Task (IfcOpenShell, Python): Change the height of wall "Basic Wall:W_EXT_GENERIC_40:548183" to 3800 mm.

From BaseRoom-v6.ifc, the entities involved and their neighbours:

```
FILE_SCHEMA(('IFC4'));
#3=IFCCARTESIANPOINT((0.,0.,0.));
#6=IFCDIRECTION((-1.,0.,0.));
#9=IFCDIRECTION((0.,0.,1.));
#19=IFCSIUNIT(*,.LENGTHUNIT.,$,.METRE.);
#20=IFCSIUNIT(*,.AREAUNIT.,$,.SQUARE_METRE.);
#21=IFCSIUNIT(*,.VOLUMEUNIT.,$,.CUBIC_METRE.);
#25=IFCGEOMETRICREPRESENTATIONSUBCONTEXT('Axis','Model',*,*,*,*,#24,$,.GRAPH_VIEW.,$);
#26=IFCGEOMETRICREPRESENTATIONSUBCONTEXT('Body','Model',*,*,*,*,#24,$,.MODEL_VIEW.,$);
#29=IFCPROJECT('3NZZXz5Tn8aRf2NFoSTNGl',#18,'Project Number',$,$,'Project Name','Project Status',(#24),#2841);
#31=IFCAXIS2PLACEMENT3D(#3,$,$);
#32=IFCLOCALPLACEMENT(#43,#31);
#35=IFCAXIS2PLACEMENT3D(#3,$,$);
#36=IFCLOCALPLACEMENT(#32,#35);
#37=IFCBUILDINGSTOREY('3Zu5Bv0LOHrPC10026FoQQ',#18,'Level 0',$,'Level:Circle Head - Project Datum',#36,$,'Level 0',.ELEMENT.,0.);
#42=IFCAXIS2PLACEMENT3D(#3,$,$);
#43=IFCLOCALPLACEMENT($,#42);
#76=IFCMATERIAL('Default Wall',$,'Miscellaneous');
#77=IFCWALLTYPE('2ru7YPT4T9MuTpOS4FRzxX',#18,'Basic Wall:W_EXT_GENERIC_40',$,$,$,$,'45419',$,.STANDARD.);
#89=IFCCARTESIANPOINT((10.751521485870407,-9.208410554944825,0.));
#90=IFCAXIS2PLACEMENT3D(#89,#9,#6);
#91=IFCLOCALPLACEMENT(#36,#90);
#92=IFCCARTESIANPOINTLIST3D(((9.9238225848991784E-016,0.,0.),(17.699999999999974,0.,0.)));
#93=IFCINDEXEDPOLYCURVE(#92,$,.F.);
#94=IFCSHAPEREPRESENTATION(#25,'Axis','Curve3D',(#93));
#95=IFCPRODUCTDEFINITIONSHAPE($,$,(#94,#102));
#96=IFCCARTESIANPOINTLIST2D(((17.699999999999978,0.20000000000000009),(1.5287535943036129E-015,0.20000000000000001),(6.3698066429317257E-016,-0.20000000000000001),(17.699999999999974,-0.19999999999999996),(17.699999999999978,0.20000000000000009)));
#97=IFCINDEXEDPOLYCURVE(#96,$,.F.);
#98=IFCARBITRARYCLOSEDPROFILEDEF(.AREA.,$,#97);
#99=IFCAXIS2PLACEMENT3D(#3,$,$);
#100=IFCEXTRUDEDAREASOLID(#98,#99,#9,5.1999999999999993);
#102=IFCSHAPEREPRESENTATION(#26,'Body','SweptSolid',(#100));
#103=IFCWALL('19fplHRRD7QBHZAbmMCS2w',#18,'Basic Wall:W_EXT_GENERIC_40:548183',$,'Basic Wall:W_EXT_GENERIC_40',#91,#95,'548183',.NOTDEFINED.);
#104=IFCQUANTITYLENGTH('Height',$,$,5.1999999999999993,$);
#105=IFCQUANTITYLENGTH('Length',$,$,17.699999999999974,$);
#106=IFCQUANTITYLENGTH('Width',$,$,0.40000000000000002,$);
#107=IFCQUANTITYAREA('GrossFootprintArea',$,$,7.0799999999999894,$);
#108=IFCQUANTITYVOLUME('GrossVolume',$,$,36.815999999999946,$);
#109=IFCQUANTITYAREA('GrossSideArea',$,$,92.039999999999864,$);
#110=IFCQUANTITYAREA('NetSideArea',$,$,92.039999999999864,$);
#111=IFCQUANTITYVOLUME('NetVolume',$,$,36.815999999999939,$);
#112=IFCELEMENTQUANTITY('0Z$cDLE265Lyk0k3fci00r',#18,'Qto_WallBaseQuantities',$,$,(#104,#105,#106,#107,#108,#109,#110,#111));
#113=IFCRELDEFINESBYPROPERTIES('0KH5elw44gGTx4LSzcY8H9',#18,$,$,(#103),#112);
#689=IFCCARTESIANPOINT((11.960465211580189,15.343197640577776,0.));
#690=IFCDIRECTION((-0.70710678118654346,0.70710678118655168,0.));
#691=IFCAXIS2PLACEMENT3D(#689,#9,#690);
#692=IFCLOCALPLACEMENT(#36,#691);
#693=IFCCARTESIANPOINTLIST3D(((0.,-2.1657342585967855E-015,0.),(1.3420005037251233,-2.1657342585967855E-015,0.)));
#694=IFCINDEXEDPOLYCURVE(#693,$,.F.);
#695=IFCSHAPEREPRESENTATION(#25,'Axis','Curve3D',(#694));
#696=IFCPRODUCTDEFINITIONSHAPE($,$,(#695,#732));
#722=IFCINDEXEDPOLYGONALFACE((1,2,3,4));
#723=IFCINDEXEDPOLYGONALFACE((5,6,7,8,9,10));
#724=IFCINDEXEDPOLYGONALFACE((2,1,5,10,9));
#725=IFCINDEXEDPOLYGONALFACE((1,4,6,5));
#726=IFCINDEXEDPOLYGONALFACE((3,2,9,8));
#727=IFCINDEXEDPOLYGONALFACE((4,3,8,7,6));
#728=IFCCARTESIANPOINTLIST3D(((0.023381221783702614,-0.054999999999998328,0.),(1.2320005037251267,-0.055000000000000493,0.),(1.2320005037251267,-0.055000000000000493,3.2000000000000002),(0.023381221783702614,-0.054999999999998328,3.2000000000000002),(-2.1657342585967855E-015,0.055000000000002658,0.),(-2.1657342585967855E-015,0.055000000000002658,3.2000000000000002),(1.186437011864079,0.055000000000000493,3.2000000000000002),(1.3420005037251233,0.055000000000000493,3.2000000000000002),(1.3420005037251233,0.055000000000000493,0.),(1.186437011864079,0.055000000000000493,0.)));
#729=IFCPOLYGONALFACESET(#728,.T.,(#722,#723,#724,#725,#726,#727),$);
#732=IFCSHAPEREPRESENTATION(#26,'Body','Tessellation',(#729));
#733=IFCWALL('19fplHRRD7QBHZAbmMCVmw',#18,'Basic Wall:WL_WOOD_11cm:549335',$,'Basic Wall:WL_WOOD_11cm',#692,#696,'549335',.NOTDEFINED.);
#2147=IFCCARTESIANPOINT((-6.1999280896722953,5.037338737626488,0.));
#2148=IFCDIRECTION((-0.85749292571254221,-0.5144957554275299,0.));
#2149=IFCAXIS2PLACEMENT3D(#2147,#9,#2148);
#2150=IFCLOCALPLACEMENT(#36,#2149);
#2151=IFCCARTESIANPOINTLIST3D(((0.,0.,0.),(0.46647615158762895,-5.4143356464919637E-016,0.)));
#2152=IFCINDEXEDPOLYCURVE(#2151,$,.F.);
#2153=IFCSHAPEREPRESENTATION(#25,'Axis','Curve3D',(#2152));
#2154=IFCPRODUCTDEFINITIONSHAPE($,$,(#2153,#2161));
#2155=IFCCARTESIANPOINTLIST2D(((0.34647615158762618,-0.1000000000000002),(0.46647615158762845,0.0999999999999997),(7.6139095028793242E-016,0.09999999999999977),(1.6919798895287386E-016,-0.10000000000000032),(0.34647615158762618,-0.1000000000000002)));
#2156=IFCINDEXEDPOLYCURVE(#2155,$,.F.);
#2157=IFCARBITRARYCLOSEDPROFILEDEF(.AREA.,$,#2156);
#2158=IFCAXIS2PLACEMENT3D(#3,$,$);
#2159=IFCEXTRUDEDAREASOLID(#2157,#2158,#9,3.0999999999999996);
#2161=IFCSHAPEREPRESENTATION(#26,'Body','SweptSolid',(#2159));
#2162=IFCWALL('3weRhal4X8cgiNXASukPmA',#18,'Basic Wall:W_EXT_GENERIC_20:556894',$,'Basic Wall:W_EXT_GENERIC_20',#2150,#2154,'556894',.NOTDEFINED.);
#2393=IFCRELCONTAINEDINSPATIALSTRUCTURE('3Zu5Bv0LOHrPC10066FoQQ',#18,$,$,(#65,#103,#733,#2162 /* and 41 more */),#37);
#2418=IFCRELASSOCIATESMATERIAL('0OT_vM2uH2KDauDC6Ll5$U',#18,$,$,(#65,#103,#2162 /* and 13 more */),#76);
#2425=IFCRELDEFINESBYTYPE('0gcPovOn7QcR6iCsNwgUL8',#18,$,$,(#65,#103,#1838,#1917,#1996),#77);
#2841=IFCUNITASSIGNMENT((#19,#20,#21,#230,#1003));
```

```python
import ifcopenshell
import ifcopenshell.api.pset
import ifcopenshell.geom
import ifcopenshell.util.element
import ifcopenshell.util.representation
import ifcopenshell.util.shape
import ifcopenshell.util.unit

model = ifcopenshell.open("BaseRoom-v6.ifc")
unit_scale = ifcopenshell.util.unit.calculate_unit_scale(model)
area_scale = ifcopenshell.util.unit.calculate_unit_scale(model, "AREAUNIT")
volume_scale = ifcopenshell.util.unit.calculate_unit_scale(model, "VOLUMEUNIT")
settings = ifcopenshell.geom.settings()


def volume(element):
    """Net volume in cubic metres, openings subtracted."""
    shape = ifcopenshell.geom.create_shape(settings, element)
    return ifcopenshell.util.shape.get_volume(shape.geometry)


wall = model.by_guid("19fplHRRD7QBHZAbmMCS2w")
before = volume(wall)

body = ifcopenshell.util.representation.get_representation(wall, "Model", "Body")
solid = body.Items[0]
old_height = solid.Depth
solid.Depth = 3.8 / unit_scale
after = volume(wall)
thickness = 0.4  # wall thickness in metres

# Update the stored height, areas and volumes.
qto = model.by_id(ifcopenshell.util.element.get_pset(wall, "Qto_WallBaseQuantities", should_inherit=False)["id"])
ifcopenshell.api.pset.edit_qto(model, qto=qto, properties={
    "Height": solid.Depth,
    "GrossVolume": ifcopenshell.util.element.get_pset(wall, "Qto_WallBaseQuantities", "GrossVolume") * solid.Depth / old_height,
    "GrossSideArea": ifcopenshell.util.element.get_pset(wall, "Qto_WallBaseQuantities", "GrossSideArea") * solid.Depth / old_height,
    "NetSideArea": after / thickness / area_scale,
    "NetVolume": after / volume_scale,
})

print(f"height {old_height:g} -> {solid.Depth:g}, volume {before:.3f} -> {after:.3f} m3")

model.write("BaseRoom-v6-out.ifc")
```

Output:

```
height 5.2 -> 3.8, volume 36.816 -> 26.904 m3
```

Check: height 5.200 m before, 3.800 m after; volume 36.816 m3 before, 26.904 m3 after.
